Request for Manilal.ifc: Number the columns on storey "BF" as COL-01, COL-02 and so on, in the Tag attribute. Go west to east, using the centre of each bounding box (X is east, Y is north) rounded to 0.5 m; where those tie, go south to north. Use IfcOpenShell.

First a look at what the model holds.

```python
import ifcopenshell
import ifcopenshell.util.element
import ifcopenshell.util.placement

model = ifcopenshell.open("Manilal.ifc")
print(model.schema)
storey = next(s for s in model.by_type("IfcBuildingStorey") if s.Name == "BF")
columns = [e for e in ifcopenshell.util.element.get_decomposition(storey) if e.is_a("IfcColumn")]
for e in sorted(columns, key=lambda e: e.id()):
    origin = ifcopenshell.util.placement.get_local_placement(e.ObjectPlacement)[:3, 3]
    print(e.id(), e.Tag, e.Name, origin.round(2) + 0.0, sep=" | ")
```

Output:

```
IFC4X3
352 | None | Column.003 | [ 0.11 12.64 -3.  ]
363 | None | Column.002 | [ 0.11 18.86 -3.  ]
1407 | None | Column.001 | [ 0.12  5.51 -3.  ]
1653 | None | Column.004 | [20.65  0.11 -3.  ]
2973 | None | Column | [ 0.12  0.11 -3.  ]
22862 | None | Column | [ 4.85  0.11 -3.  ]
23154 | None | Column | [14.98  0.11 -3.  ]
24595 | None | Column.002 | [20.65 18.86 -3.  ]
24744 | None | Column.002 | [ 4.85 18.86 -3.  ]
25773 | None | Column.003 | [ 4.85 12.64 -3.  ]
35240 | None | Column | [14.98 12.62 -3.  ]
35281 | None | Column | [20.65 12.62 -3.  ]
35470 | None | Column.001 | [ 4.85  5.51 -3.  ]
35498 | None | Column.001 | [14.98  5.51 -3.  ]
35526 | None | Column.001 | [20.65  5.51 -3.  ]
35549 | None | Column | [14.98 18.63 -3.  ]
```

```python
import ifcopenshell
import ifcopenshell.geom
import ifcopenshell.util.element
import ifcopenshell.util.shape

model = ifcopenshell.open("Manilal.ifc")
settings = ifcopenshell.geom.settings()
settings.set("use-world-coords", True)


def centre(element):
    shape = ifcopenshell.geom.create_shape(settings, element)
    return ifcopenshell.util.shape.get_bbox_centroid(shape.geometry)


storey = next(s for s in model.by_type("IfcBuildingStorey") if s.Name == "BF")
columns = [e for e in ifcopenshell.util.element.get_decomposition(storey) if e.is_a("IfcColumn")]

# Insertion points can sit at a corner or the storey origin, so sort by the geometry (in metres).
centres = {e: centre(e) for e in columns}
columns.sort(key=lambda e: (round(centres[e][0] / 0.5), centres[e][1]))

for i, e in enumerate(columns, start=1):
    number = f"COL-{i:02d}"
    e.Tag = number
    print(e.id(), number)

model.write("Manilal_updated.ifc")
```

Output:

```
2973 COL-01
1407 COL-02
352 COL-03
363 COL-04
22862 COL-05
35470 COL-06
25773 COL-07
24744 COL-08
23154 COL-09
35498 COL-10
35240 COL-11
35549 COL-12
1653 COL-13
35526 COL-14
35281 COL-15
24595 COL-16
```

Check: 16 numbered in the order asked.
